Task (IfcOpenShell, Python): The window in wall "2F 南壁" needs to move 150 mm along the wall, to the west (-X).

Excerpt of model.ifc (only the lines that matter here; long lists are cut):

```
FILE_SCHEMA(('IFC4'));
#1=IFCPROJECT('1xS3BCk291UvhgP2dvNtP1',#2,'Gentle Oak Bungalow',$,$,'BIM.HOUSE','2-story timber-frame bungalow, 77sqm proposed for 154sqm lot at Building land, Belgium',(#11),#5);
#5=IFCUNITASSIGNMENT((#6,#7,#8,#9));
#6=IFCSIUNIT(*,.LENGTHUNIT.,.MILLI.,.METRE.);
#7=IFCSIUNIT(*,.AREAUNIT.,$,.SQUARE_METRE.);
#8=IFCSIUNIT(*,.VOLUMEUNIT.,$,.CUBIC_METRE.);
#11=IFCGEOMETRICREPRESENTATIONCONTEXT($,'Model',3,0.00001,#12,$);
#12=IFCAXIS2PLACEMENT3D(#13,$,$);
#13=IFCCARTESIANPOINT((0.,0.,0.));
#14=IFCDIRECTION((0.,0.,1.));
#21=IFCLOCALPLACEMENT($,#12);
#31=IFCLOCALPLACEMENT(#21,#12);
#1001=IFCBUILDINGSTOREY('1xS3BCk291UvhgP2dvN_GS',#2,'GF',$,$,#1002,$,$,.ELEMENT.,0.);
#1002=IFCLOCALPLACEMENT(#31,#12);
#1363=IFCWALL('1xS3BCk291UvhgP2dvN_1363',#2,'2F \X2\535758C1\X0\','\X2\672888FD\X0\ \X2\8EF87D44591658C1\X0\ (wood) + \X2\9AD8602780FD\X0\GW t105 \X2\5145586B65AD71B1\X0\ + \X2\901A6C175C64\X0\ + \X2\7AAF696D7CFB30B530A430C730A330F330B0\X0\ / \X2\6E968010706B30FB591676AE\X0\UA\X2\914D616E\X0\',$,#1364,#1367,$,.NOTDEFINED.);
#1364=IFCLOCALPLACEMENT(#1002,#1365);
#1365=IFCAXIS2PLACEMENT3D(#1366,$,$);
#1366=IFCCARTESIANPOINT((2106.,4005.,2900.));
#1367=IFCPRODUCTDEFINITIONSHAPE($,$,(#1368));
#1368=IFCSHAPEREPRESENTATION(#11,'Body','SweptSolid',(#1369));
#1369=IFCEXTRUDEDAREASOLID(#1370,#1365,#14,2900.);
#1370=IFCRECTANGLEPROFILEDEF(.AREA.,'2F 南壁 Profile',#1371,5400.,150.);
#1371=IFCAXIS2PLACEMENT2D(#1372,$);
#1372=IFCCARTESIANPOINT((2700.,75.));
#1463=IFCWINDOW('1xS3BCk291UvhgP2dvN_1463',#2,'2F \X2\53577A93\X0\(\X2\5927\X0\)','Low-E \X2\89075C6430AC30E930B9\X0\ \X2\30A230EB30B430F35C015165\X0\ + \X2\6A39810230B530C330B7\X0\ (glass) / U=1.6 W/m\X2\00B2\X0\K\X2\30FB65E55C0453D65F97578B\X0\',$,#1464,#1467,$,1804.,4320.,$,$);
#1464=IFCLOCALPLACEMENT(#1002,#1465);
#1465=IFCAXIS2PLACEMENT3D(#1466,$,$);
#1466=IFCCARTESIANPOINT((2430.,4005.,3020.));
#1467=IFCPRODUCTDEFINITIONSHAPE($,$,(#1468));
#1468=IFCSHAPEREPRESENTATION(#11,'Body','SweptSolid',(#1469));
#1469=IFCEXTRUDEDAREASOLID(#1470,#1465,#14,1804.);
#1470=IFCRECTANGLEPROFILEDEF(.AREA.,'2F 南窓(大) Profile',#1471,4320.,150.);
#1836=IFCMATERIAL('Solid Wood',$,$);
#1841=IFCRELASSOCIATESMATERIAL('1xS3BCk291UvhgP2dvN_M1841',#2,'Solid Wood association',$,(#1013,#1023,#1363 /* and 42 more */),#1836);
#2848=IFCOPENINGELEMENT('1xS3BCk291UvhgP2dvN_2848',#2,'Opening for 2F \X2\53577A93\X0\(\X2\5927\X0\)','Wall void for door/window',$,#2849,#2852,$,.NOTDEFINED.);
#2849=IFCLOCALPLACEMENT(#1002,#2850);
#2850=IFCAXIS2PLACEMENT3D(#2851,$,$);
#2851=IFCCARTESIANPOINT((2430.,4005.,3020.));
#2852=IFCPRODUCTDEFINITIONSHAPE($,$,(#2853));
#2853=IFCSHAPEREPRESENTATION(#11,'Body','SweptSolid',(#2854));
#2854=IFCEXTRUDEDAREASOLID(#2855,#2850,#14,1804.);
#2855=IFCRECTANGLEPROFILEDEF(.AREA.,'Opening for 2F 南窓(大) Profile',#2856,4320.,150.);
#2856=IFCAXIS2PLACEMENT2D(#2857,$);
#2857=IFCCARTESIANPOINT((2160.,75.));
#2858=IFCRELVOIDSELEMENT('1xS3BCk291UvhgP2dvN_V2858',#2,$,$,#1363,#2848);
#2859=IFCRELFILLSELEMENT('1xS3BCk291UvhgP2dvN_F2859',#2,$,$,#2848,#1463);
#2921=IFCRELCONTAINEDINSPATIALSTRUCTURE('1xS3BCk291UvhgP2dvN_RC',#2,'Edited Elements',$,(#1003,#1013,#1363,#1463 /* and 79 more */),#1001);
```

```python
import ifcopenshell
import ifcopenshell.api.geometry
import ifcopenshell.util.placement
import ifcopenshell.util.unit

model = ifcopenshell.open("model.ifc")
unit_scale = ifcopenshell.util.unit.calculate_unit_scale(model)

window = model.by_guid("1xS3BCk291UvhgP2dvN_1463")
opening = window.FillsVoids[0].RelatingOpeningElement
wall = opening.VoidsElements[0].RelatingBuildingElement

wall_matrix = ifcopenshell.util.placement.get_local_placement(wall.ObjectPlacement)
shift = wall_matrix[:3, 0] * -0.15 / unit_scale
before = ifcopenshell.util.placement.get_local_placement(window.ObjectPlacement)[:3, 3].copy()

# The window is not placed relative to its opening, so move both.
for product in (opening, window):
    matrix = ifcopenshell.util.placement.get_local_placement(product.ObjectPlacement)
    matrix[:3, 3] += shift
    ifcopenshell.api.geometry.edit_object_placement(model, product=product, matrix=matrix, is_si=False)

after = ifcopenshell.util.placement.get_local_placement(window.ObjectPlacement)[:3, 3]
print("window moved by", (after - before).round(3) + 0.0)

model.write("model-out.ifc")
```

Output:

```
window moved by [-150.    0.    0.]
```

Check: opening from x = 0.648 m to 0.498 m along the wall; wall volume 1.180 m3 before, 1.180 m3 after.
